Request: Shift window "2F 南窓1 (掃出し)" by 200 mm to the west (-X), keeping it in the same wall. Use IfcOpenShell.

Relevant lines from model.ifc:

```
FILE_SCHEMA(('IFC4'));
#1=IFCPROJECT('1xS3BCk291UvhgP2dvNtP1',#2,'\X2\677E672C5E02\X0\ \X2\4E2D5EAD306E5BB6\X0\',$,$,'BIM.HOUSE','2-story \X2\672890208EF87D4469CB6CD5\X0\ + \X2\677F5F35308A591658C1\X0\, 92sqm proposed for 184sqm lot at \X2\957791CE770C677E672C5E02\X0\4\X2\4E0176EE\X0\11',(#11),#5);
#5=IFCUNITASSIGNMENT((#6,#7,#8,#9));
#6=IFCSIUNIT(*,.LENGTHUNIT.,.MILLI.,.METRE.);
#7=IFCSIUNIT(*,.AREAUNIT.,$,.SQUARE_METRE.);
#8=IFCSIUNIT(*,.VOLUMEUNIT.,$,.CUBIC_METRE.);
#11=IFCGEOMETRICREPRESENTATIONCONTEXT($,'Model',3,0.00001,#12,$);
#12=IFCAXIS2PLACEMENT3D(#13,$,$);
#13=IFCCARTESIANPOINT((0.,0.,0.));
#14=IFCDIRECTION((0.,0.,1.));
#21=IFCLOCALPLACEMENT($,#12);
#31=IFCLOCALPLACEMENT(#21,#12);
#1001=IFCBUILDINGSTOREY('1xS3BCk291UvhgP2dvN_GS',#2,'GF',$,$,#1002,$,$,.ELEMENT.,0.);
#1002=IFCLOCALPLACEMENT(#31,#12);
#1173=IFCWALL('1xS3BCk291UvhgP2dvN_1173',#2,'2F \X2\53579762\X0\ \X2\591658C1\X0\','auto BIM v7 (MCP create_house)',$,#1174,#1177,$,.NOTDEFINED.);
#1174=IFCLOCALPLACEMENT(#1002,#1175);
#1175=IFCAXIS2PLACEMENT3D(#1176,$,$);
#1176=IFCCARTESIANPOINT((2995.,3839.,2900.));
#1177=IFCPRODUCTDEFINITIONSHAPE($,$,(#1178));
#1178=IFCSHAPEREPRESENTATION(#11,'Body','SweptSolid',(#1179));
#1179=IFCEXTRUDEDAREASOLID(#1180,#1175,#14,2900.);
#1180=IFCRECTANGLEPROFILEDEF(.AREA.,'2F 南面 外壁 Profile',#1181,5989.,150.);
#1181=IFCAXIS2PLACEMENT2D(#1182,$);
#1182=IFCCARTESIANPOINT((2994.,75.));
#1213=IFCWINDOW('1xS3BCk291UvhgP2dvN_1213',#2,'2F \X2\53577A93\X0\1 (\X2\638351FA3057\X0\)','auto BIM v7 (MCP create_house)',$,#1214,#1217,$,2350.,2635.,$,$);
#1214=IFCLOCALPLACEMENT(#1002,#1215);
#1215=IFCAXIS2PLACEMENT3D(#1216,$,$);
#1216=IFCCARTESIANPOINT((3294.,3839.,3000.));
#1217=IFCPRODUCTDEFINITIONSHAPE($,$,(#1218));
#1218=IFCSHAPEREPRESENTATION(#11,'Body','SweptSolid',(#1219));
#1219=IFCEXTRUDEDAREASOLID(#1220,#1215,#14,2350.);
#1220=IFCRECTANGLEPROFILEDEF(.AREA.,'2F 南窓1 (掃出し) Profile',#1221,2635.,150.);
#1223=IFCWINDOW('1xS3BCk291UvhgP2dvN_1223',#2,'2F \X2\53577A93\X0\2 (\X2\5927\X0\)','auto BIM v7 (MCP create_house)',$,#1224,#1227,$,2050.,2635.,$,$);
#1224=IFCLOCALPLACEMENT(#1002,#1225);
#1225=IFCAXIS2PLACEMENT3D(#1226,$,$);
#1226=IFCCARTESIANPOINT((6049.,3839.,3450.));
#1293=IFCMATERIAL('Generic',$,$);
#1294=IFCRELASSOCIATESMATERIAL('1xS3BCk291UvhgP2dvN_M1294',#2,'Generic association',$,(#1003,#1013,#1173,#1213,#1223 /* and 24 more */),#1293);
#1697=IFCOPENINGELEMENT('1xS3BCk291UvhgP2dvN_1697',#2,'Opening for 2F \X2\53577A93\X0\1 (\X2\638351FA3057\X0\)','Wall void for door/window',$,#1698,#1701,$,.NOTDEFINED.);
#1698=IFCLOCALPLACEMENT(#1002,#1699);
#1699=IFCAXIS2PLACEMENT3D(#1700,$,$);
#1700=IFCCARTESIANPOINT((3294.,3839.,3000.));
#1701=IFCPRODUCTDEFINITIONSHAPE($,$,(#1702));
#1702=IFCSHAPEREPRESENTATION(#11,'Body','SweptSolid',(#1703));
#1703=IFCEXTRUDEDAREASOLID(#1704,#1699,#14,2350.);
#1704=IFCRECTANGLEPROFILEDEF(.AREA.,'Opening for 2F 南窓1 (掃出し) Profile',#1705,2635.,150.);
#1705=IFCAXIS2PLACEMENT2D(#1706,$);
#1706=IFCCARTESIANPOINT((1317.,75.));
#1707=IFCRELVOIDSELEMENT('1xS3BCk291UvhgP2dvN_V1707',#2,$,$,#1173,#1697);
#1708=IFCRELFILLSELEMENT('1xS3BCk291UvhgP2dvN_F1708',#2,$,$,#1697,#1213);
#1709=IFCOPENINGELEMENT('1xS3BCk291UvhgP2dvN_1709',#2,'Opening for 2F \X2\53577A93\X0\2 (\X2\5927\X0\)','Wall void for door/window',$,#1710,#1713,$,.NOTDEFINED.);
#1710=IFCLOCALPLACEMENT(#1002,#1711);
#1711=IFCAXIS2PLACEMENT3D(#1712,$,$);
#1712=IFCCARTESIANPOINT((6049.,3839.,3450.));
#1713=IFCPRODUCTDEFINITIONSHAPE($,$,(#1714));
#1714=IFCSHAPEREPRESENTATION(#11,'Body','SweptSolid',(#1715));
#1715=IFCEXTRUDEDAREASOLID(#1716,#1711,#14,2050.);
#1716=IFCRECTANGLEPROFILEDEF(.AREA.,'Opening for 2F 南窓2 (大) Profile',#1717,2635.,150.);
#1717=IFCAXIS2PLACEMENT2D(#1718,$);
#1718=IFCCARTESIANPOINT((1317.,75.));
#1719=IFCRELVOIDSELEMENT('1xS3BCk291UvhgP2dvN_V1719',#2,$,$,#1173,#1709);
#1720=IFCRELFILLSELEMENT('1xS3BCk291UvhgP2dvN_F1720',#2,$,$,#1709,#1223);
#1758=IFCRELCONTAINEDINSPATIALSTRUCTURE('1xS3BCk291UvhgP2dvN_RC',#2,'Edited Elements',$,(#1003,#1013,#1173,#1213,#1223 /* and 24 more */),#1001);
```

```python
import ifcopenshell
import ifcopenshell.api.geometry
import ifcopenshell.util.placement
import ifcopenshell.util.unit

model = ifcopenshell.open("model.ifc")
unit_scale = ifcopenshell.util.unit.calculate_unit_scale(model)

window = model.by_guid("1xS3BCk291UvhgP2dvN_1213")
opening = window.FillsVoids[0].RelatingOpeningElement
wall = opening.VoidsElements[0].RelatingBuildingElement

wall_matrix = ifcopenshell.util.placement.get_local_placement(wall.ObjectPlacement)
shift = wall_matrix[:3, 0] * -0.2 / unit_scale
before = ifcopenshell.util.placement.get_local_placement(window.ObjectPlacement)[:3, 3].copy()

# The window is not placed relative to its opening, so move both.
for product in (opening, window):
    matrix = ifcopenshell.util.placement.get_local_placement(product.ObjectPlacement)
    matrix[:3, 3] += shift
    ifcopenshell.api.geometry.edit_object_placement(model, product=product, matrix=matrix, is_si=False)

after = ifcopenshell.util.placement.get_local_placement(window.ObjectPlacement)[:3, 3]
print("window moved by", (after - before).round(3) + 0.0)

model.write("model_rev.ifc")
```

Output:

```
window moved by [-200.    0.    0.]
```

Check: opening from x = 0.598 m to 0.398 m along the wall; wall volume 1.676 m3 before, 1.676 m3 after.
